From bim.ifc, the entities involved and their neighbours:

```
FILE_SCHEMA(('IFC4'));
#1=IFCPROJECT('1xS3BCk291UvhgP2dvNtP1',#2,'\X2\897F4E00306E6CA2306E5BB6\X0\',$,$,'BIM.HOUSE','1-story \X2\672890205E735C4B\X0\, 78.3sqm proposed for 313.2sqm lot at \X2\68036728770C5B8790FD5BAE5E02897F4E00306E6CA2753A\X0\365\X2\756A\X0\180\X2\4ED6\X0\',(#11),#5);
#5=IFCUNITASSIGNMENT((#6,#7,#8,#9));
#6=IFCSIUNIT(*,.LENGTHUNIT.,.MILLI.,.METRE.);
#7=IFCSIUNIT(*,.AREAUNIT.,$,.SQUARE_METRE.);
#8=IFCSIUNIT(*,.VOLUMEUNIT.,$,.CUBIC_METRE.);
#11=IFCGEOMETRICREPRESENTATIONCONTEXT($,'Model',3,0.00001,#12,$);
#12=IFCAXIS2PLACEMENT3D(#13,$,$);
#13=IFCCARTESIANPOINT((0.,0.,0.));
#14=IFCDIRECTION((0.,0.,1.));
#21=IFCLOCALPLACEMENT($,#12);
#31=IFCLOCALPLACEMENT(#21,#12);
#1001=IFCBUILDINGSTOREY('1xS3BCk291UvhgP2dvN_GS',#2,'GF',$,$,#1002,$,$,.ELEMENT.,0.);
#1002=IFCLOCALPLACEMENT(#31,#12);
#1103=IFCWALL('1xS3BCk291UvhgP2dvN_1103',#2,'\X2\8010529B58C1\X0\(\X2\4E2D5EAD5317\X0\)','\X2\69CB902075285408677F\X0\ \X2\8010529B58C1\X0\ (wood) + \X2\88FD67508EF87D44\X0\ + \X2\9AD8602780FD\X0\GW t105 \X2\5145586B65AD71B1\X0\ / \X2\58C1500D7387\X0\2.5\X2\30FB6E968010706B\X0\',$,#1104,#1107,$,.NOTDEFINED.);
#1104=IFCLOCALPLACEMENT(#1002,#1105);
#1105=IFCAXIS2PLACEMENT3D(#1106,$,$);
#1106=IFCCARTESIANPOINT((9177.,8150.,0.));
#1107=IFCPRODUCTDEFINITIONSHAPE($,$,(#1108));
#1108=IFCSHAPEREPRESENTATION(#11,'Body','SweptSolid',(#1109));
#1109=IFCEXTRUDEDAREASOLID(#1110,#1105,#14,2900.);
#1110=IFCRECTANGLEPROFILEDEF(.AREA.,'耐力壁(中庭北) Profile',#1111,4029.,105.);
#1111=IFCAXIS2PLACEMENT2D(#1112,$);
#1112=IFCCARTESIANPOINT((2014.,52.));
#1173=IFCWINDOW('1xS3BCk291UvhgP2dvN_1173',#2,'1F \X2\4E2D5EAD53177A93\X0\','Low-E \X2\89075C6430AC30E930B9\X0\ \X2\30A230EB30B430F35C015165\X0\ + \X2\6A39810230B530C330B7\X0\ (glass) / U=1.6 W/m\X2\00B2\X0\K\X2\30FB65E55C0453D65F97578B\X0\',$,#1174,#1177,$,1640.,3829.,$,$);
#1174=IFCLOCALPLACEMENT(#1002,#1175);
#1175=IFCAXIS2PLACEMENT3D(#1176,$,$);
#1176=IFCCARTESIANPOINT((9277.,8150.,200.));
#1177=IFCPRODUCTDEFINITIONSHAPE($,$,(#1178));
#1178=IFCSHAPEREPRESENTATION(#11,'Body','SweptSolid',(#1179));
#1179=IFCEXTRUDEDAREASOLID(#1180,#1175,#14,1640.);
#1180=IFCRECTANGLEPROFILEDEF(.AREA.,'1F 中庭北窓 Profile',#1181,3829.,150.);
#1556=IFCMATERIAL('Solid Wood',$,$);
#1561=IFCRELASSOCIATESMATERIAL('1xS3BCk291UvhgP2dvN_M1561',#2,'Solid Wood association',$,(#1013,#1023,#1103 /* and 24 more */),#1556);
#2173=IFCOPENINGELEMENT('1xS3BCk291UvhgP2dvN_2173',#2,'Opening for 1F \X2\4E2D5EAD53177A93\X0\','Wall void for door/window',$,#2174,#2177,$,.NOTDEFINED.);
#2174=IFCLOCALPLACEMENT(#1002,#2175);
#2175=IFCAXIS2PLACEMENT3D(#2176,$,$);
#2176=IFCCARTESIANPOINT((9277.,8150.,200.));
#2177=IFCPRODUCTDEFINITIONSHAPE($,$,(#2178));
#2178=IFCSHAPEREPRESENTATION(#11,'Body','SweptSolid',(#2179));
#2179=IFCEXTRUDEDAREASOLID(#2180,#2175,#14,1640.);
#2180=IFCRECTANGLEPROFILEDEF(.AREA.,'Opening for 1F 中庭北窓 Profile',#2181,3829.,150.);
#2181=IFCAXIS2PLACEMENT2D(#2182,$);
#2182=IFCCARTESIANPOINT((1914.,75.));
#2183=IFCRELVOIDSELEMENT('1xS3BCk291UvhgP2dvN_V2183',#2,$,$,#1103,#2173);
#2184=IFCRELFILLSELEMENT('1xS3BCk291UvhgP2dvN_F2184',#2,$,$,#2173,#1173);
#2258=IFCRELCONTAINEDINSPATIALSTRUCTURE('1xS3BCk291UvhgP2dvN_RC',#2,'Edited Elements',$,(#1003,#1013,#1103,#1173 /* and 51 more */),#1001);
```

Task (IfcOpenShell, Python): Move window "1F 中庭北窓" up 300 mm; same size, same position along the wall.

```python
import numpy as np
import ifcopenshell
import ifcopenshell.api.geometry
import ifcopenshell.util.placement
import ifcopenshell.util.unit

model = ifcopenshell.open("bim.ifc")
unit_scale = ifcopenshell.util.unit.calculate_unit_scale(model)

window = model.by_id(1173)
opening = window.FillsVoids[0].RelatingOpeningElement
dz = 0.3 / unit_scale

shift = np.array([0.0, 0.0, dz])
# The window is not placed relative to its opening, so move both.
for product in (opening, window):
    matrix = ifcopenshell.util.placement.get_local_placement(product.ObjectPlacement)
    matrix[:3, 3] += shift
    ifcopenshell.api.geometry.edit_object_placement(model, product=product, matrix=matrix, is_si=False)

print(f"moved by {dz * unit_scale:+.3f} m")

model.write("bim_rev.ifc")
```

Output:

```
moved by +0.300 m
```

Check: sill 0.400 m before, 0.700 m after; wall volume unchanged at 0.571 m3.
